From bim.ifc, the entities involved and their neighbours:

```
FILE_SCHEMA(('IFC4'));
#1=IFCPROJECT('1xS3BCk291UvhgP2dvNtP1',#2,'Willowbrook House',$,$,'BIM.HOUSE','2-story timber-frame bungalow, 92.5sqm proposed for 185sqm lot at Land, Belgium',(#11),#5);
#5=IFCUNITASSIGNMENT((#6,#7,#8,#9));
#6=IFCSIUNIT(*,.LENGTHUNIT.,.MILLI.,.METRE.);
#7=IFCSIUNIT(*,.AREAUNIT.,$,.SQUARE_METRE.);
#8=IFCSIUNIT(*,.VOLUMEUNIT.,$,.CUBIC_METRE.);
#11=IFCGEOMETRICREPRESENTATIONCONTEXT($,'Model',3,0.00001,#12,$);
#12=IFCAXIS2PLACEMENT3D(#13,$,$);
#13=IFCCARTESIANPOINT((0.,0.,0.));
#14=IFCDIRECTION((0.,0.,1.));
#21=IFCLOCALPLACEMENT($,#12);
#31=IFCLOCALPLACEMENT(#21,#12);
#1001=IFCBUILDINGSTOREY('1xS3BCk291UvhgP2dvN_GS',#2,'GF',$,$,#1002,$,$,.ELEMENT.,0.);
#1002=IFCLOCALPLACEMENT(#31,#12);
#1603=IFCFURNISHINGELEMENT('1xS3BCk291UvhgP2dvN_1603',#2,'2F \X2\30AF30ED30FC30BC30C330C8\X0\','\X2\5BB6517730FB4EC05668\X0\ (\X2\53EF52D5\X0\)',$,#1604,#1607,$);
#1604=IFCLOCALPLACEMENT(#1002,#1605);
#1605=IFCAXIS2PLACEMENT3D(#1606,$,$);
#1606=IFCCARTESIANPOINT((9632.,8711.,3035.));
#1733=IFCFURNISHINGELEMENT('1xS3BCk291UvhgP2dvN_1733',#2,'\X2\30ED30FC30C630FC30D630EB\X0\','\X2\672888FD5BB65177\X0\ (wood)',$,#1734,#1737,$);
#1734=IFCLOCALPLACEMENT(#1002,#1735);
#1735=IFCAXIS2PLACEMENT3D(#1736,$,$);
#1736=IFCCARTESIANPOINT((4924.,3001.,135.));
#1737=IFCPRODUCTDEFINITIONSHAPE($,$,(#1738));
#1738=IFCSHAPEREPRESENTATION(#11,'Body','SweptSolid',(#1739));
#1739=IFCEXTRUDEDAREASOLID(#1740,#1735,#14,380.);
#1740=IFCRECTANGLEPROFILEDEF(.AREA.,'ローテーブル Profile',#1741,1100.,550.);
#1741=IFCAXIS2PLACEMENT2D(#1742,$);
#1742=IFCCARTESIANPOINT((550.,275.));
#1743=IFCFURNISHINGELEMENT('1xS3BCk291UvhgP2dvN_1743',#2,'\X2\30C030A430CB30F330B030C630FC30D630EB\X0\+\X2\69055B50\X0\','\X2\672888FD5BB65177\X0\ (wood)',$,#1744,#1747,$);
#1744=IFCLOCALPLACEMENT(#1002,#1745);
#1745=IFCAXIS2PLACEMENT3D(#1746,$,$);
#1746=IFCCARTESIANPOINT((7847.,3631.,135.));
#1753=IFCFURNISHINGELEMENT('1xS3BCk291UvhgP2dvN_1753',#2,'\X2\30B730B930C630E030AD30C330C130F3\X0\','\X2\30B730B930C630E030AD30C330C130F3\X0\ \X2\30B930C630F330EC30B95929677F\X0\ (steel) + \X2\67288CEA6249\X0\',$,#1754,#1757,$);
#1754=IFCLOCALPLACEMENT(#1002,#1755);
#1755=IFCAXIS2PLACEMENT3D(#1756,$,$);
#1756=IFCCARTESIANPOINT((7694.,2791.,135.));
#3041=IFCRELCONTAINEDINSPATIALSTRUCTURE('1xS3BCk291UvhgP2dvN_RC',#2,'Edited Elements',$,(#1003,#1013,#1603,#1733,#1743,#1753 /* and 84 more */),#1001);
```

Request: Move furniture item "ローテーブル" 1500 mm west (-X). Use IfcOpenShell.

```python
import ifcopenshell
import ifcopenshell.api.geometry
import ifcopenshell.util.placement

model = ifcopenshell.open("bim.ifc")

item = model.by_guid("1xS3BCk291UvhgP2dvN_1733")
matrix = ifcopenshell.util.placement.get_local_placement(item.ObjectPlacement)
matrix[0, 3] -= 1500.0
ifcopenshell.api.geometry.edit_object_placement(model, product=item, matrix=matrix, is_si=False)

print(ifcopenshell.util.placement.get_local_placement(item.ObjectPlacement).round(3) + 0.0)

model.write("bim_v2.ifc")
```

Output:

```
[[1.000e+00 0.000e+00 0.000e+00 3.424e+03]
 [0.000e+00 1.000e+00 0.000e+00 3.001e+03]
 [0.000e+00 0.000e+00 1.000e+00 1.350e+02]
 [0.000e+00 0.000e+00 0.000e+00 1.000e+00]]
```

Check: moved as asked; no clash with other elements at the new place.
